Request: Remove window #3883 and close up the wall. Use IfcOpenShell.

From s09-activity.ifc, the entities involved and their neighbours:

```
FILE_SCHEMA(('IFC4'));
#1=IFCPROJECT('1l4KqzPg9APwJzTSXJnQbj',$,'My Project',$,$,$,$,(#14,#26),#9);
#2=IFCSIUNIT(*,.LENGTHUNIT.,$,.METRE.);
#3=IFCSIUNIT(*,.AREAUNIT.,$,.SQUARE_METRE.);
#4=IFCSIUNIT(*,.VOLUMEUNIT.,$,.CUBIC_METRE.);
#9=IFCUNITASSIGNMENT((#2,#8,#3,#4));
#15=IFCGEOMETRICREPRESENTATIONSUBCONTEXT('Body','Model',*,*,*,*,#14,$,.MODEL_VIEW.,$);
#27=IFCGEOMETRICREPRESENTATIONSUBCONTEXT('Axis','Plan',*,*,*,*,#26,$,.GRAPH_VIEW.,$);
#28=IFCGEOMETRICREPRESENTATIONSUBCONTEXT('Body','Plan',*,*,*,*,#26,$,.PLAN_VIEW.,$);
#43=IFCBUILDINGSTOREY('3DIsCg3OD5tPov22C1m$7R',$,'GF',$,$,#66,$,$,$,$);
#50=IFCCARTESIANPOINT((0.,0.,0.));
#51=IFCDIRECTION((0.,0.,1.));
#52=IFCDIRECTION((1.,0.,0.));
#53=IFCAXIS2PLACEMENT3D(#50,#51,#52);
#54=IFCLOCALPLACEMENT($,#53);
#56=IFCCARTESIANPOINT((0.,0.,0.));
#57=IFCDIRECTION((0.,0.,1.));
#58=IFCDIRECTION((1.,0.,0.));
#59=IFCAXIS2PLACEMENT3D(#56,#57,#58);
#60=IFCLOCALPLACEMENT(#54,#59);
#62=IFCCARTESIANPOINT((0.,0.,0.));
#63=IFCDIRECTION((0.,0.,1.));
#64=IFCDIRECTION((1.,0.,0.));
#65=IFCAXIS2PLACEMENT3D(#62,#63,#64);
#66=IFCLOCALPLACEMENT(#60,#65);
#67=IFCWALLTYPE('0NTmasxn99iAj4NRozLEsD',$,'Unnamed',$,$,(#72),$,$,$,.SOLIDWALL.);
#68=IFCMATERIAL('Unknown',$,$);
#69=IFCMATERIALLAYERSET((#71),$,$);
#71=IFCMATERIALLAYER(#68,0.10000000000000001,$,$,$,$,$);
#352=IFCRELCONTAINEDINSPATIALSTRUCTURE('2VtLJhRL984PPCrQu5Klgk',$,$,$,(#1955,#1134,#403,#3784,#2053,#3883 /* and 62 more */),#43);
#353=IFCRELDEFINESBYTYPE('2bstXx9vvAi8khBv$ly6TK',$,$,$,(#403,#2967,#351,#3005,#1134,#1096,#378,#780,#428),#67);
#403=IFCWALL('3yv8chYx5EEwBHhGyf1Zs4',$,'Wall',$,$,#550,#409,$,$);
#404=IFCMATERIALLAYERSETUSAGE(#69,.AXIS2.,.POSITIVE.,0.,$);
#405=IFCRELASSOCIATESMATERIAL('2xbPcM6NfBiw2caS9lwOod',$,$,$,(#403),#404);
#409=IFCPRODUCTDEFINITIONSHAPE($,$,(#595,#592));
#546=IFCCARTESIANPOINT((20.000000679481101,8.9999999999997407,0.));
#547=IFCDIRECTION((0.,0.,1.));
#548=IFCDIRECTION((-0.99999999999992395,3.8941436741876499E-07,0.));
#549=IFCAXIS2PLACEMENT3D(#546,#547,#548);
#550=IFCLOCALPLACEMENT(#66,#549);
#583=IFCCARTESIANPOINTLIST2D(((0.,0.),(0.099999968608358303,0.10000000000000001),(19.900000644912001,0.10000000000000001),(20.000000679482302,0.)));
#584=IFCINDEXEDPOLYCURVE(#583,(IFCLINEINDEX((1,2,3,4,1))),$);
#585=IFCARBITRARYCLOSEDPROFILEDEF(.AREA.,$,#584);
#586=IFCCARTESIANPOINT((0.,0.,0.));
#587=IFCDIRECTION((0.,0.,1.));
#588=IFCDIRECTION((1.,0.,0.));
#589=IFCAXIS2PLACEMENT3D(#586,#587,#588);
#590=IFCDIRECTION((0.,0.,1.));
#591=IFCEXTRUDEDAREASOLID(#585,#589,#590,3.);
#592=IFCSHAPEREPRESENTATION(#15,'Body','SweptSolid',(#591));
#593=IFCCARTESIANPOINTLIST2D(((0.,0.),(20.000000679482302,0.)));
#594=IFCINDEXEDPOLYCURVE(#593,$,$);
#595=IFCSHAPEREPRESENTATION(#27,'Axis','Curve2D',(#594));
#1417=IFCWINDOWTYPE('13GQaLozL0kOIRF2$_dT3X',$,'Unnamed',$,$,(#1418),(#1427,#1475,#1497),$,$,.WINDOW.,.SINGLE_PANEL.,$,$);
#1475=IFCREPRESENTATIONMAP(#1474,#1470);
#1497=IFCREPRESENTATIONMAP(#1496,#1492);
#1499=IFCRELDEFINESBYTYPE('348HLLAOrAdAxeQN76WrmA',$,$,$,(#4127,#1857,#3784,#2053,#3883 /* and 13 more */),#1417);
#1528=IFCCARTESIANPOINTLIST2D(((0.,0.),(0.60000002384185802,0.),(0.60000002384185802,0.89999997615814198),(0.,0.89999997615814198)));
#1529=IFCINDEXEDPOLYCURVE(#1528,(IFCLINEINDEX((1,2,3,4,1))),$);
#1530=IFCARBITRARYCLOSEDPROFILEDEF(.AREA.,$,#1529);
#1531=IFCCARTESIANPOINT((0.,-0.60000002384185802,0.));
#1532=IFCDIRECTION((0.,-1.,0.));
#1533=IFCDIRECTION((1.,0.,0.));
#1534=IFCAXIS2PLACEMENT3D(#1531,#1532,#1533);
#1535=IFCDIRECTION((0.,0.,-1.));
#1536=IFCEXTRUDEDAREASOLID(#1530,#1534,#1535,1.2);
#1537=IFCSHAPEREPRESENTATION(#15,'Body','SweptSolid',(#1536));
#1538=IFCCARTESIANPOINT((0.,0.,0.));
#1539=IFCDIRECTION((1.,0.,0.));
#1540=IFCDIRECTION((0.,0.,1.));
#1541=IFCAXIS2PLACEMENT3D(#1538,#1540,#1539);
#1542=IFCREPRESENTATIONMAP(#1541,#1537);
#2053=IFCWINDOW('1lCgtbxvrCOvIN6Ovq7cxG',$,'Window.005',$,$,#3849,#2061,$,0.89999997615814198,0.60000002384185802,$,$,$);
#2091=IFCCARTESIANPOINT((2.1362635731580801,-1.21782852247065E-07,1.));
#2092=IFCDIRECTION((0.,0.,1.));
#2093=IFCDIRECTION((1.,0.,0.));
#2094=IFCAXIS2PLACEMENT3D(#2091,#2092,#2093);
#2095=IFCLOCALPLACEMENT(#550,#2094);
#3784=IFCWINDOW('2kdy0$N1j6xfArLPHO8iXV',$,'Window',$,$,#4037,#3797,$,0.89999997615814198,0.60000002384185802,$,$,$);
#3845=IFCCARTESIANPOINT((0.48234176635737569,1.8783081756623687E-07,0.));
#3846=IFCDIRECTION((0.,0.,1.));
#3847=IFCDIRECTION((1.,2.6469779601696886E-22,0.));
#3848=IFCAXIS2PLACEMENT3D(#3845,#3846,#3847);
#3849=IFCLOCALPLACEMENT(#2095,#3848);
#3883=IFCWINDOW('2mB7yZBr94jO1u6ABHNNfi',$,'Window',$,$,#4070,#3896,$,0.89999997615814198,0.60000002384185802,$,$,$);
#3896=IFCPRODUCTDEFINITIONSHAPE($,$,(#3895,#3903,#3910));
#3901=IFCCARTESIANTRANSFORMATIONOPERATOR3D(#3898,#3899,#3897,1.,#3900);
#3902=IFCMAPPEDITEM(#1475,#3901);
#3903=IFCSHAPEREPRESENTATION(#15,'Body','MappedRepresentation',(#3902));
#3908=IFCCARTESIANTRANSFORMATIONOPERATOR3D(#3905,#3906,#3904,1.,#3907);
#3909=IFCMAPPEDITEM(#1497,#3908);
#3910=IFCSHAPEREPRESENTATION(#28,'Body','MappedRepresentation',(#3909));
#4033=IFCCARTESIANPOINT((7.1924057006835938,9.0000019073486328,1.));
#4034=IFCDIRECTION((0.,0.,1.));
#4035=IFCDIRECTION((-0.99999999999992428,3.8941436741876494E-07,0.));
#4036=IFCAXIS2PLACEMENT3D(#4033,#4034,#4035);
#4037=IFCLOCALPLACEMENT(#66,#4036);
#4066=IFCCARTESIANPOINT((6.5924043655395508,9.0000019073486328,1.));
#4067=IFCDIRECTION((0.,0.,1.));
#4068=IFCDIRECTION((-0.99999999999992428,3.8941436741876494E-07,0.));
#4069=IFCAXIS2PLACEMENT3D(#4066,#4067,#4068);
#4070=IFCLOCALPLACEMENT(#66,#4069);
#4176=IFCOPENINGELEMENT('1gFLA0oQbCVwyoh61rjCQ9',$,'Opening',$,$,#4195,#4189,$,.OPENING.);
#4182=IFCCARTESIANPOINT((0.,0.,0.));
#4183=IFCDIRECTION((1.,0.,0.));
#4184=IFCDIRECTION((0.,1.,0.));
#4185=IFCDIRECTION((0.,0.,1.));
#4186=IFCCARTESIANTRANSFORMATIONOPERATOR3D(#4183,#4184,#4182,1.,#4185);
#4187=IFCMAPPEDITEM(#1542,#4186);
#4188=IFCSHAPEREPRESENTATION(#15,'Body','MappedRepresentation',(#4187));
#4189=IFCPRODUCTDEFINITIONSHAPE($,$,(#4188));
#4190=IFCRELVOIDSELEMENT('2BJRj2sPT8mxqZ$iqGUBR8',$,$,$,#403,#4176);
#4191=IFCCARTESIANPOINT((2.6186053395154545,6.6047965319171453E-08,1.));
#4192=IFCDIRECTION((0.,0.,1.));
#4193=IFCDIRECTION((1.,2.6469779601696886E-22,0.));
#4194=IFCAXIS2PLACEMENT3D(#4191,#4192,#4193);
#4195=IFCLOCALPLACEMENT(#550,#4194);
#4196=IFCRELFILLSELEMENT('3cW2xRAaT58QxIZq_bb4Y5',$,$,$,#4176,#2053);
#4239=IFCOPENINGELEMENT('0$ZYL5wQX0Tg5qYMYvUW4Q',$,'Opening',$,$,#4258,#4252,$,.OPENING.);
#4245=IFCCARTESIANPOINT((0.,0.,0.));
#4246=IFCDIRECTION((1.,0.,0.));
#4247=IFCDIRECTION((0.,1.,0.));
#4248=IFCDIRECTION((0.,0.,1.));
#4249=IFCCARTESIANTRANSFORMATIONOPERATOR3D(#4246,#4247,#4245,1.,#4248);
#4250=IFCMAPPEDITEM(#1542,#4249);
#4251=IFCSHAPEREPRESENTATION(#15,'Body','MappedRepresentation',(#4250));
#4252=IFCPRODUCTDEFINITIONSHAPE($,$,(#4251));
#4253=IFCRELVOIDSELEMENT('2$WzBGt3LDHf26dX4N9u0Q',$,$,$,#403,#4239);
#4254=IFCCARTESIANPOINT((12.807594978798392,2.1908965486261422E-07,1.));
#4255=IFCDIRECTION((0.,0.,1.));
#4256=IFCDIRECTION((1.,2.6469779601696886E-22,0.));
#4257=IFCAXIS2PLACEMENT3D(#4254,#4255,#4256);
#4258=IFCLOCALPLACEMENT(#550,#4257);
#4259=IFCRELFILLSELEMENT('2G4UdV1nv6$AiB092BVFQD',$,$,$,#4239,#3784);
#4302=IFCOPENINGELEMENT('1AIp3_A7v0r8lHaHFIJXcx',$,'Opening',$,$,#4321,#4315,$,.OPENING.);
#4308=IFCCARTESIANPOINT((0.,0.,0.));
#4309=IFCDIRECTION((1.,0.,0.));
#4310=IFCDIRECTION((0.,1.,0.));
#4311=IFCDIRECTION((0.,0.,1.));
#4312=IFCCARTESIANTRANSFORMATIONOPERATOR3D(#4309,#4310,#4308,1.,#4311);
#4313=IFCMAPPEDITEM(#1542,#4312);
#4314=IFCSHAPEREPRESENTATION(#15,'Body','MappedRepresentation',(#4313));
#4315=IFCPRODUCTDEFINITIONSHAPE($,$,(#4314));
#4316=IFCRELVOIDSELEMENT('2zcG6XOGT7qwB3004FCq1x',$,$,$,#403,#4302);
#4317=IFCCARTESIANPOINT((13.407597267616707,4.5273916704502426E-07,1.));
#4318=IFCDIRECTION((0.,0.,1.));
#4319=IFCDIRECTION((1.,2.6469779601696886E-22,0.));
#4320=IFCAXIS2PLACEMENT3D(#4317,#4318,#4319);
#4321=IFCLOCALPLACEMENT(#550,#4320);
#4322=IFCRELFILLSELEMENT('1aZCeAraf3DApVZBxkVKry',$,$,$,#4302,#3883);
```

```python
import ifcopenshell
import ifcopenshell.api.feature
import ifcopenshell.api.root
import ifcopenshell.geom
import ifcopenshell.util.shape

model = ifcopenshell.open("s09-activity.ifc")
settings = ifcopenshell.geom.settings()


def volume(element):
    """Net volume in cubic metres, openings subtracted."""
    shape = ifcopenshell.geom.create_shape(settings, element)
    return ifcopenshell.util.shape.get_volume(shape.geometry)


window = model.by_id(3883)
opening = window.FillsVoids[0].RelatingOpeningElement
wall = opening.VoidsElements[0].RelatingBuildingElement
before = volume(wall)

ifcopenshell.api.root.remove_product(model, product=window)
ifcopenshell.api.feature.remove_feature(model, feature=opening)

after = volume(wall)

print(f"wall volume {before:.3f} -> {after:.3f} m3")

model.write("s09-activity_rev.ifc")
```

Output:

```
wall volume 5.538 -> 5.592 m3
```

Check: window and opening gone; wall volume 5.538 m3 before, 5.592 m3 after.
